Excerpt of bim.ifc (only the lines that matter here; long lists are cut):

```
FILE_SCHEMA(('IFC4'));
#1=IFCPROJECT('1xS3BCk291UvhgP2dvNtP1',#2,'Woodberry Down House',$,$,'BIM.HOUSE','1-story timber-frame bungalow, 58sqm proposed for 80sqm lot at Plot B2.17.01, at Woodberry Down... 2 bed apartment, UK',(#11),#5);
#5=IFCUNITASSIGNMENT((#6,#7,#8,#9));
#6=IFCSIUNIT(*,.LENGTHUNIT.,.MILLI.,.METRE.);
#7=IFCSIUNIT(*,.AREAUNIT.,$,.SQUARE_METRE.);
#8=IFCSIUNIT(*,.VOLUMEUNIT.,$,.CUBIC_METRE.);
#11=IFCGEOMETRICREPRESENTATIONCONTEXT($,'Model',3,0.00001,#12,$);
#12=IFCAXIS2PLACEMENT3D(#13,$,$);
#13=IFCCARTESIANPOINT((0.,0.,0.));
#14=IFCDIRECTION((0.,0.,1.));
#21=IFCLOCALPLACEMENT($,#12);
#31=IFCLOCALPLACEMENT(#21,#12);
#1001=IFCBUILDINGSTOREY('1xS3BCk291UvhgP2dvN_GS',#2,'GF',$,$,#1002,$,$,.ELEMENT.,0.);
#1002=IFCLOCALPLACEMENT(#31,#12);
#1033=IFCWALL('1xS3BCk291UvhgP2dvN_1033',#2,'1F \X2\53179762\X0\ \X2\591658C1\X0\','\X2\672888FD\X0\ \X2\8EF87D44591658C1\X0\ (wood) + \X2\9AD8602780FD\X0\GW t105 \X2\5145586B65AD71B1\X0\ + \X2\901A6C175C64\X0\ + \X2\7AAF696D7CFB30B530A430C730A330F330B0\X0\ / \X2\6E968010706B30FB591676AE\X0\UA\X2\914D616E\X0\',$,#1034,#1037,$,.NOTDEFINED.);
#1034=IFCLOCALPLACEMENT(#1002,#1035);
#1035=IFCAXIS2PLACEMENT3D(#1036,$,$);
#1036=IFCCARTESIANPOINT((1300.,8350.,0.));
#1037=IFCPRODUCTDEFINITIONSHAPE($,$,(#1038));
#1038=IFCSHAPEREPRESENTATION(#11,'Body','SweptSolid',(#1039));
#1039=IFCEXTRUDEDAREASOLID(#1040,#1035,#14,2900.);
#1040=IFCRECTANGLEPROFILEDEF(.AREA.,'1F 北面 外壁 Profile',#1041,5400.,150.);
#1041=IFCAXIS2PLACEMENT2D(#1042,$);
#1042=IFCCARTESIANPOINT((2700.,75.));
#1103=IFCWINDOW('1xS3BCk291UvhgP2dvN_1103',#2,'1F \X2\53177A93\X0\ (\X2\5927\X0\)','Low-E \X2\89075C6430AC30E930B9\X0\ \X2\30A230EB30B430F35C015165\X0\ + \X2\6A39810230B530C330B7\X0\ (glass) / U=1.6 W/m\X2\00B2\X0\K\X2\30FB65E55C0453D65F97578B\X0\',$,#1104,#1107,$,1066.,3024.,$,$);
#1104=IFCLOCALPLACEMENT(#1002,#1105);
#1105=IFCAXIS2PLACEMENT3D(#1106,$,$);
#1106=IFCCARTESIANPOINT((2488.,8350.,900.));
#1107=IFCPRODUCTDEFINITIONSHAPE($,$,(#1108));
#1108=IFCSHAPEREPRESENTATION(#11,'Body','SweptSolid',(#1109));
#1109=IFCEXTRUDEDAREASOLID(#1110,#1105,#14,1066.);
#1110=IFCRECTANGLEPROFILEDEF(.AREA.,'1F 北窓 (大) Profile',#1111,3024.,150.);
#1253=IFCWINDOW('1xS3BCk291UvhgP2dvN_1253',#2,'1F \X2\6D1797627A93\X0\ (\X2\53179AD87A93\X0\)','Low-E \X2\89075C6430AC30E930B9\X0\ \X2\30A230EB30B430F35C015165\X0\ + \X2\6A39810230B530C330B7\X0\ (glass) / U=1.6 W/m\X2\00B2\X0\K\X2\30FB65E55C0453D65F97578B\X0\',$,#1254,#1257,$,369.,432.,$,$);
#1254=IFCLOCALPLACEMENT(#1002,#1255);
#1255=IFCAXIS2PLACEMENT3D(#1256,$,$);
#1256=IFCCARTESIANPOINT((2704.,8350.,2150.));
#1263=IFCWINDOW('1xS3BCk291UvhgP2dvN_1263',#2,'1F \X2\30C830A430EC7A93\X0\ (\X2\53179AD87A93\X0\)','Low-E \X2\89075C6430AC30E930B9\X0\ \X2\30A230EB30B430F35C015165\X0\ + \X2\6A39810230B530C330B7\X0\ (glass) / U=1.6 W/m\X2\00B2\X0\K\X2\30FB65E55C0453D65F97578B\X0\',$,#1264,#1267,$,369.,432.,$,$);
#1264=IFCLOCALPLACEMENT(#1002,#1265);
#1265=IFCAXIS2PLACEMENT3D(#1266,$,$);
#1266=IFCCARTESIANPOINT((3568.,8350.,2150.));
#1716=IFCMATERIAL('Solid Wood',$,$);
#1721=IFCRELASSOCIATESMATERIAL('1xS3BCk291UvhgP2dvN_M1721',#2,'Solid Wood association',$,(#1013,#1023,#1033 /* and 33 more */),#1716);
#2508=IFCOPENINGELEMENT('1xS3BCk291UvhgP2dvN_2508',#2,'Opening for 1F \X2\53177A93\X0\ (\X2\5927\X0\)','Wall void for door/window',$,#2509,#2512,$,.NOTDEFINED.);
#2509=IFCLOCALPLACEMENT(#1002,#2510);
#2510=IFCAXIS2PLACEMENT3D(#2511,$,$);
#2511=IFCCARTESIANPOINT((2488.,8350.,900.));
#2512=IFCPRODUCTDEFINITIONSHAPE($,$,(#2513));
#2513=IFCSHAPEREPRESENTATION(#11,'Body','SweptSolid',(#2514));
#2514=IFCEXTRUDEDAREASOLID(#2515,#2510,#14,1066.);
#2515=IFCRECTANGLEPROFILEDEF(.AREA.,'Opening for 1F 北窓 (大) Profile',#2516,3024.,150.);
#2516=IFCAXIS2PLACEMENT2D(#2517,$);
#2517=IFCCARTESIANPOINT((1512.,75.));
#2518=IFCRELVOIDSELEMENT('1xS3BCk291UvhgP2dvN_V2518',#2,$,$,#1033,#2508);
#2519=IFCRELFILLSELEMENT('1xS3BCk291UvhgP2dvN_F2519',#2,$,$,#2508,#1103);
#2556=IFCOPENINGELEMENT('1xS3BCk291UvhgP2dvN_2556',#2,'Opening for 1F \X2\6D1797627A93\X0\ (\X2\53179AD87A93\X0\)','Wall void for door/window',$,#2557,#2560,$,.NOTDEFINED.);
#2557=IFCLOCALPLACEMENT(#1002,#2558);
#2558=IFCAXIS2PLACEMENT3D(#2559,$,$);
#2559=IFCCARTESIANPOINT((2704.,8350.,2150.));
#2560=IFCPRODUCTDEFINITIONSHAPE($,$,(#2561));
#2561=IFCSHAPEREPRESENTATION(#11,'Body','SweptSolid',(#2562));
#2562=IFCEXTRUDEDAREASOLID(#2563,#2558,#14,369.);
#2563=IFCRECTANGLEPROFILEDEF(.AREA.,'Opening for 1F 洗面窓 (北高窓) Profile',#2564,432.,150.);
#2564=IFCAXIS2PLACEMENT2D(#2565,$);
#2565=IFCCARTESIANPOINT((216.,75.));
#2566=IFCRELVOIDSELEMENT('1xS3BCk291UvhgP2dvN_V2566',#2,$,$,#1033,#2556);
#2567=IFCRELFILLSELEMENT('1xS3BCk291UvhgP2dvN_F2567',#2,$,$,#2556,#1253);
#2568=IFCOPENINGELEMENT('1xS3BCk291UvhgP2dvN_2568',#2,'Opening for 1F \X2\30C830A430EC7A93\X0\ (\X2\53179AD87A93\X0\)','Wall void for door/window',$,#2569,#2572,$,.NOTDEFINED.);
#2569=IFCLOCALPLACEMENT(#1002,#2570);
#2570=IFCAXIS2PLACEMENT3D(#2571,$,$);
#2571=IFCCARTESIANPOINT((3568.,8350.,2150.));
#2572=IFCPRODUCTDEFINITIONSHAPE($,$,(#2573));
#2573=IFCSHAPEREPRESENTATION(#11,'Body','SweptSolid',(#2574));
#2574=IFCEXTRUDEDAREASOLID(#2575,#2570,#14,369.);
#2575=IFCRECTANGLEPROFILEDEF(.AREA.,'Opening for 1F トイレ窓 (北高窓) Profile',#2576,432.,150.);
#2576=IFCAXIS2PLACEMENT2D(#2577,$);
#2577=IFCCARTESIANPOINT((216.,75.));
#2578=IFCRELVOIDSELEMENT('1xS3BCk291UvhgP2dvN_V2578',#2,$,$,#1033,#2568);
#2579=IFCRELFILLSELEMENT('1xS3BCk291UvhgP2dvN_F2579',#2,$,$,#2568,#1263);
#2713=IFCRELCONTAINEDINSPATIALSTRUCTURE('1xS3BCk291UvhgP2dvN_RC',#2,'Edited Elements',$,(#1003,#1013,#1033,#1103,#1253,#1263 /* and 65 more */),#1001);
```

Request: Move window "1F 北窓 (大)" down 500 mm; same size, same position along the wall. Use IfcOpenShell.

```python
import numpy as np
import ifcopenshell
import ifcopenshell.api.geometry
import ifcopenshell.util.placement
import ifcopenshell.util.unit

model = ifcopenshell.open("bim.ifc")
unit_scale = ifcopenshell.util.unit.calculate_unit_scale(model)

window = model.by_guid("1xS3BCk291UvhgP2dvN_1103")
opening = window.FillsVoids[0].RelatingOpeningElement
dz = -0.5 / unit_scale

shift = np.array([0.0, 0.0, dz])
# The window is not placed relative to its opening, so move both.
for product in (opening, window):
    matrix = ifcopenshell.util.placement.get_local_placement(product.ObjectPlacement)
    matrix[:3, 3] += shift
    ifcopenshell.api.geometry.edit_object_placement(model, product=product, matrix=matrix, is_si=False)

print(f"moved by {dz * unit_scale:+.3f} m")

model.write("bim_updated.ifc")
```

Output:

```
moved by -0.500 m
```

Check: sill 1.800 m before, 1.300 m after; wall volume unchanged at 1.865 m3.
